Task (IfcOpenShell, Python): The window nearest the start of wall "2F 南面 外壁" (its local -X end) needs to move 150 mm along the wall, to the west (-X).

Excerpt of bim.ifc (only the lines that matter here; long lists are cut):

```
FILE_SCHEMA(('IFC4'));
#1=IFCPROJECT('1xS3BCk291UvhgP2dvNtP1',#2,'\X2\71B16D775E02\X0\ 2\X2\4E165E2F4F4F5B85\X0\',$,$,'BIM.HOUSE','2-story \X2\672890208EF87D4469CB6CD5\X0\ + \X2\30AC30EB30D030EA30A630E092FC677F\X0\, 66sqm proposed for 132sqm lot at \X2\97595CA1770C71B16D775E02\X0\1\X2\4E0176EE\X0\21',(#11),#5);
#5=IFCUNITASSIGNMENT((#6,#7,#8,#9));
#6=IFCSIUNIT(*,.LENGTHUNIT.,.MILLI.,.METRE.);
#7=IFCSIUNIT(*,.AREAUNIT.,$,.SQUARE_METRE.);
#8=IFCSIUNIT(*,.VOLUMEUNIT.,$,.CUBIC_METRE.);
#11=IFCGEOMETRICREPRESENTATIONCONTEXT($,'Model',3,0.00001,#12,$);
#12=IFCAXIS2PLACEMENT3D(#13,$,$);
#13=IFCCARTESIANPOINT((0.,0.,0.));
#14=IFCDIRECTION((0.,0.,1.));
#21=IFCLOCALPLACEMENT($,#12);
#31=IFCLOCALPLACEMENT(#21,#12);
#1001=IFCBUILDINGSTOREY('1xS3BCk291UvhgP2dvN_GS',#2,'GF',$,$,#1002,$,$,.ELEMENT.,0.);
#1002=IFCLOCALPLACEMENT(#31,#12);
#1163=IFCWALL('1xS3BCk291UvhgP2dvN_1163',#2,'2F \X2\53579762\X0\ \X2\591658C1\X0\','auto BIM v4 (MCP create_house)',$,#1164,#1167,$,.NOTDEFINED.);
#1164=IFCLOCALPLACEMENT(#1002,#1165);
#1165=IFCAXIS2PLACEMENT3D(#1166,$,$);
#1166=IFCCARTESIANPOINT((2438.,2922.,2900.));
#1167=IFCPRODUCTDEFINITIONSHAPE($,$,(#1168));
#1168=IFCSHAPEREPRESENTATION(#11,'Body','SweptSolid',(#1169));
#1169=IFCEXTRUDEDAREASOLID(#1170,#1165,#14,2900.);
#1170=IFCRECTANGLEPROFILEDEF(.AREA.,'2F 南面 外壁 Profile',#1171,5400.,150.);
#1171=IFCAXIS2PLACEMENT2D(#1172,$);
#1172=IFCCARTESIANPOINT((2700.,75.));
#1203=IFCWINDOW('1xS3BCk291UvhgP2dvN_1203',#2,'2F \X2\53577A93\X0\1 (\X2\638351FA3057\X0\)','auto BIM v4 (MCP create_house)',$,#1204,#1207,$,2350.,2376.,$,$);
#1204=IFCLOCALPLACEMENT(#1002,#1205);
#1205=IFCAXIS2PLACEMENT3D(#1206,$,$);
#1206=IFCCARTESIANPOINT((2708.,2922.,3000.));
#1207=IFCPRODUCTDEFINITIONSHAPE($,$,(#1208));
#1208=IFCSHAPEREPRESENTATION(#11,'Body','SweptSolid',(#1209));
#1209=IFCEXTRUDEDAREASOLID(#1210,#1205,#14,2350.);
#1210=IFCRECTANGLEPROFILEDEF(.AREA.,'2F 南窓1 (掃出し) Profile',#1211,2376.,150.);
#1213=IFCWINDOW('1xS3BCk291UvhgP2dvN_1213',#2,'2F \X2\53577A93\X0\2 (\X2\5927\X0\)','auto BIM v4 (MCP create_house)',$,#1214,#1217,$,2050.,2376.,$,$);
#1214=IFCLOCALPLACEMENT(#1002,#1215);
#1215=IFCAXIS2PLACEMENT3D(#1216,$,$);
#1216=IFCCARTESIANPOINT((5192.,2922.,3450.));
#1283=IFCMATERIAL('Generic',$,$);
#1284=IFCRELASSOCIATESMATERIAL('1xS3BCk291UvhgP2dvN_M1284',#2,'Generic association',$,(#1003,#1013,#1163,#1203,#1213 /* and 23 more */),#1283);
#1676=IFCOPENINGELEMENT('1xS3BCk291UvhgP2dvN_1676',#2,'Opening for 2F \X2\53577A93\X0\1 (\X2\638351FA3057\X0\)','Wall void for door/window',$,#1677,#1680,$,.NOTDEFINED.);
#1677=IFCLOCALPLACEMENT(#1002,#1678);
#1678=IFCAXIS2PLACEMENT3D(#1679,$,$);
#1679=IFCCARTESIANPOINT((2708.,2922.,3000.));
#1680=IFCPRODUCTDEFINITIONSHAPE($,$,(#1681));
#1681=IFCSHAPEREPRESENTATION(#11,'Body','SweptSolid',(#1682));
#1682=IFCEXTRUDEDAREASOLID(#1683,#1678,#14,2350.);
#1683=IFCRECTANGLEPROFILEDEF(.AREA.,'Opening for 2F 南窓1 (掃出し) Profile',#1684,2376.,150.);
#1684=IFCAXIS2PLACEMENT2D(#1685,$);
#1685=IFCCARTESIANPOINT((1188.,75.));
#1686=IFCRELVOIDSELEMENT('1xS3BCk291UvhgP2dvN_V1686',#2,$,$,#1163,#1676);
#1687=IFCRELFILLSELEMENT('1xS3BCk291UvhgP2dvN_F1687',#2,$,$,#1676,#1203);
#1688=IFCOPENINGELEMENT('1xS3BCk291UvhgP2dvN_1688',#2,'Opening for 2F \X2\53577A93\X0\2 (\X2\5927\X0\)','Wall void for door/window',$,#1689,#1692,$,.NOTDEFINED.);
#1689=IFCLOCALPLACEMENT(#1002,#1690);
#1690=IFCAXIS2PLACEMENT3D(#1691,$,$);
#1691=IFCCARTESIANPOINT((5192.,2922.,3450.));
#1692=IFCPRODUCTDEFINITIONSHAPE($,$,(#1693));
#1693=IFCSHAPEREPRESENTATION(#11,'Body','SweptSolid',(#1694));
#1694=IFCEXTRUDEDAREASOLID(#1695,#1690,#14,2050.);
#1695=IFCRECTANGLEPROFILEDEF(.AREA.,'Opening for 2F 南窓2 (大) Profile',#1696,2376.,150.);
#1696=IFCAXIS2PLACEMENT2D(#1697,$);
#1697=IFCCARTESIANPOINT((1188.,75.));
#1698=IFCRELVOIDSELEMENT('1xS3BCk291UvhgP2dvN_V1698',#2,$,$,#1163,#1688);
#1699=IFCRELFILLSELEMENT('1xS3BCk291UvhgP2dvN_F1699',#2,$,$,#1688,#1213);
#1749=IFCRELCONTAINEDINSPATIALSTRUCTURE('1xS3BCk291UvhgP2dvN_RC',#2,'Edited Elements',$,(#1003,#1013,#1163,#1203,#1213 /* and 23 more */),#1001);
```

```python
import ifcopenshell
import ifcopenshell.api.geometry
import ifcopenshell.util.placement

model = ifcopenshell.open("bim.ifc")

window = model.by_guid("1xS3BCk291UvhgP2dvN_1203")
opening = window.FillsVoids[0].RelatingOpeningElement
wall = opening.VoidsElements[0].RelatingBuildingElement

wall_matrix = ifcopenshell.util.placement.get_local_placement(wall.ObjectPlacement)
shift = wall_matrix[:3, 0] * -150.0
before = ifcopenshell.util.placement.get_local_placement(window.ObjectPlacement)[:3, 3].copy()

# The window is not placed relative to its opening, so move both.
for product in (opening, window):
    matrix = ifcopenshell.util.placement.get_local_placement(product.ObjectPlacement)
    matrix[:3, 3] += shift
    ifcopenshell.api.geometry.edit_object_placement(model, product=product, matrix=matrix, is_si=False)

after = ifcopenshell.util.placement.get_local_placement(window.ObjectPlacement)[:3, 3]
print("window moved by", (after - before).round(3) + 0.0)

model.write("bim_edited.ifc")
```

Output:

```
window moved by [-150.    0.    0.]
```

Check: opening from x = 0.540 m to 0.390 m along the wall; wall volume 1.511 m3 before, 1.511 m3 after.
